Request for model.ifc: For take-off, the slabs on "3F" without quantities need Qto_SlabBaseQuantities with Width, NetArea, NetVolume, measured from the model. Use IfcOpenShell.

First a look at what the model holds.

```python
import ifcopenshell
import ifcopenshell.util.element
import ifcopenshell.util.unit

model = ifcopenshell.open("model.ifc")
print(model.schema)
for unit_type in ("LENGTHUNIT", "AREAUNIT", "VOLUMEUNIT"):
    print(unit_type, ifcopenshell.util.unit.calculate_unit_scale(model, unit_type))
storey = next(s for s in model.by_type("IfcBuildingStorey") if s.Name == "3F")
slabs = [e for e in ifcopenshell.util.element.get_decomposition(storey) if e.is_a("IfcSlab")]
for e in sorted(slabs, key=lambda e: e.id()):
    print(e.id(), e.is_a(), e.Name, list(ifcopenshell.util.element.get_psets(e, qtos_only=True)), sep=" | ")
```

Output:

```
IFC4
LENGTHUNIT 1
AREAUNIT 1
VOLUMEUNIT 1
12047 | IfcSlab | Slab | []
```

```python
import ifcopenshell
import ifcopenshell.api.pset
import ifcopenshell.geom
import ifcopenshell.util.element
import ifcopenshell.util.shape
import ifcopenshell.util.unit

model = ifcopenshell.open("model.ifc")
unit_scale = ifcopenshell.util.unit.calculate_unit_scale(model)
area_scale = ifcopenshell.util.unit.calculate_unit_scale(model, "AREAUNIT")
volume_scale = ifcopenshell.util.unit.calculate_unit_scale(model, "VOLUMEUNIT")
settings = ifcopenshell.geom.settings()

storey = next(s for s in model.by_type("IfcBuildingStorey") if s.Name == "3F")
slabs = [e for e in ifcopenshell.util.element.get_decomposition(storey) if e.is_a("IfcSlab")]

for e in sorted(slabs, key=lambda e: e.id()):
    if ifcopenshell.util.element.get_psets(e, qtos_only=True, should_inherit=False):
        continue
    # Geometry comes back in metres, in the element's own axes.
    shape = ifcopenshell.geom.create_shape(settings, e)
    values = {
        "Width": ifcopenshell.util.shape.get_z(shape.geometry) / unit_scale,
        "NetArea": ifcopenshell.util.shape.get_footprint_area(shape.geometry) / area_scale,
        "NetVolume": ifcopenshell.util.shape.get_volume(shape.geometry) / volume_scale,
    }
    qto = ifcopenshell.api.pset.add_qto(model, product=e, name="Qto_SlabBaseQuantities")
    ifcopenshell.api.pset.edit_qto(model, qto=qto, properties=values)
    print(e.id(), {k: round(v, 3) for k, v in values.items()})

model.write("model_updated.ifc")
```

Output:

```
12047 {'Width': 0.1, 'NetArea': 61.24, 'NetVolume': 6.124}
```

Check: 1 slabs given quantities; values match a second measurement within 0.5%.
